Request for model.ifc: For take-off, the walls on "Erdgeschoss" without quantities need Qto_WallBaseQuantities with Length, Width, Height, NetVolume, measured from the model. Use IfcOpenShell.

First a look at what the model holds.

```python
import ifcopenshell
import ifcopenshell.util.element
import ifcopenshell.util.unit

model = ifcopenshell.open("model.ifc")
print(model.schema)
for unit_type in ("LENGTHUNIT", "AREAUNIT", "VOLUMEUNIT"):
    print(unit_type, ifcopenshell.util.unit.calculate_unit_scale(model, unit_type))
storey = next(s for s in model.by_type("IfcBuildingStorey") if s.Name == "Erdgeschoss")
walls = [e for e in ifcopenshell.util.element.get_decomposition(storey) if e.is_a("IfcWall")]
for e in sorted(walls, key=lambda e: e.id()):
    print(e.id(), e.is_a(), e.Name, list(ifcopenshell.util.element.get_psets(e, qtos_only=True)), sep=" | ")
```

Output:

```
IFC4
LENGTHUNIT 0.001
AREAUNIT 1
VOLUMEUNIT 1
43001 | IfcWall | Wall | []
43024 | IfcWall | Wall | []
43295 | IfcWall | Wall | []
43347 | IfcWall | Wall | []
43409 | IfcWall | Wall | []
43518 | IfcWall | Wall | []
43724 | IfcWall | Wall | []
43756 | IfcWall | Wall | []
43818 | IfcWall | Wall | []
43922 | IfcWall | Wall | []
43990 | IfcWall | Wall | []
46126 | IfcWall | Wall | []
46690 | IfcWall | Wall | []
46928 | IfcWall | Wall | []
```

```python
import ifcopenshell
import ifcopenshell.api.pset
import ifcopenshell.geom
import ifcopenshell.util.element
import ifcopenshell.util.shape
import ifcopenshell.util.unit

model = ifcopenshell.open("model.ifc")
unit_scale = ifcopenshell.util.unit.calculate_unit_scale(model)
volume_scale = ifcopenshell.util.unit.calculate_unit_scale(model, "VOLUMEUNIT")
settings = ifcopenshell.geom.settings()

storey = next(s for s in model.by_type("IfcBuildingStorey") if s.Name == "Erdgeschoss")
walls = [e for e in ifcopenshell.util.element.get_decomposition(storey) if e.is_a("IfcWall")]

for e in sorted(walls, key=lambda e: e.id()):
    if ifcopenshell.util.element.get_psets(e, qtos_only=True, should_inherit=False):
        continue
    # Geometry comes back in metres, in the element's own axes.
    shape = ifcopenshell.geom.create_shape(settings, e)
    values = {
        "Length": ifcopenshell.util.shape.get_x(shape.geometry) / unit_scale,
        "Width": ifcopenshell.util.shape.get_y(shape.geometry) / unit_scale,
        "Height": ifcopenshell.util.shape.get_z(shape.geometry) / unit_scale,
        "NetVolume": ifcopenshell.util.shape.get_volume(shape.geometry) / volume_scale,
    }
    qto = ifcopenshell.api.pset.add_qto(model, product=e, name="Qto_WallBaseQuantities")
    ifcopenshell.api.pset.edit_qto(model, qto=qto, properties=values)
    print(e.id(), {k: round(v, 3) for k, v in values.items()})

model.write("model_v2.ifc")
```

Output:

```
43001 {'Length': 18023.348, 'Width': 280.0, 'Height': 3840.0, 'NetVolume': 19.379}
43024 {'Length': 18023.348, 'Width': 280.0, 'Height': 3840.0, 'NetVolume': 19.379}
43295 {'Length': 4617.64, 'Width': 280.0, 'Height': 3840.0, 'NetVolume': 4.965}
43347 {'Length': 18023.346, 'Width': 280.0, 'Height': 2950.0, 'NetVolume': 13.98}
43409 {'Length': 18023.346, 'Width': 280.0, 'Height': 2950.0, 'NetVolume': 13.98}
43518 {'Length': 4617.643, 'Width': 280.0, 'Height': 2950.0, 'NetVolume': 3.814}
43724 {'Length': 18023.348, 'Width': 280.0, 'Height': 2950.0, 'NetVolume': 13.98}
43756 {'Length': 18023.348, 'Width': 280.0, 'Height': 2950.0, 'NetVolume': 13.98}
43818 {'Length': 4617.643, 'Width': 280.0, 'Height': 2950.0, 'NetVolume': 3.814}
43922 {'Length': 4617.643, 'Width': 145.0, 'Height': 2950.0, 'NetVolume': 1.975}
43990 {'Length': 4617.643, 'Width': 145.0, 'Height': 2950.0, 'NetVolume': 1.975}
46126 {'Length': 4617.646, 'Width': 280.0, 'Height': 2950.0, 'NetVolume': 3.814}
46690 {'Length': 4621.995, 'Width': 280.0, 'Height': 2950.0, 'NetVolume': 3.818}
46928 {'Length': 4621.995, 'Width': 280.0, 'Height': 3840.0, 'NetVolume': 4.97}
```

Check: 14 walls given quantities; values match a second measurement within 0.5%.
